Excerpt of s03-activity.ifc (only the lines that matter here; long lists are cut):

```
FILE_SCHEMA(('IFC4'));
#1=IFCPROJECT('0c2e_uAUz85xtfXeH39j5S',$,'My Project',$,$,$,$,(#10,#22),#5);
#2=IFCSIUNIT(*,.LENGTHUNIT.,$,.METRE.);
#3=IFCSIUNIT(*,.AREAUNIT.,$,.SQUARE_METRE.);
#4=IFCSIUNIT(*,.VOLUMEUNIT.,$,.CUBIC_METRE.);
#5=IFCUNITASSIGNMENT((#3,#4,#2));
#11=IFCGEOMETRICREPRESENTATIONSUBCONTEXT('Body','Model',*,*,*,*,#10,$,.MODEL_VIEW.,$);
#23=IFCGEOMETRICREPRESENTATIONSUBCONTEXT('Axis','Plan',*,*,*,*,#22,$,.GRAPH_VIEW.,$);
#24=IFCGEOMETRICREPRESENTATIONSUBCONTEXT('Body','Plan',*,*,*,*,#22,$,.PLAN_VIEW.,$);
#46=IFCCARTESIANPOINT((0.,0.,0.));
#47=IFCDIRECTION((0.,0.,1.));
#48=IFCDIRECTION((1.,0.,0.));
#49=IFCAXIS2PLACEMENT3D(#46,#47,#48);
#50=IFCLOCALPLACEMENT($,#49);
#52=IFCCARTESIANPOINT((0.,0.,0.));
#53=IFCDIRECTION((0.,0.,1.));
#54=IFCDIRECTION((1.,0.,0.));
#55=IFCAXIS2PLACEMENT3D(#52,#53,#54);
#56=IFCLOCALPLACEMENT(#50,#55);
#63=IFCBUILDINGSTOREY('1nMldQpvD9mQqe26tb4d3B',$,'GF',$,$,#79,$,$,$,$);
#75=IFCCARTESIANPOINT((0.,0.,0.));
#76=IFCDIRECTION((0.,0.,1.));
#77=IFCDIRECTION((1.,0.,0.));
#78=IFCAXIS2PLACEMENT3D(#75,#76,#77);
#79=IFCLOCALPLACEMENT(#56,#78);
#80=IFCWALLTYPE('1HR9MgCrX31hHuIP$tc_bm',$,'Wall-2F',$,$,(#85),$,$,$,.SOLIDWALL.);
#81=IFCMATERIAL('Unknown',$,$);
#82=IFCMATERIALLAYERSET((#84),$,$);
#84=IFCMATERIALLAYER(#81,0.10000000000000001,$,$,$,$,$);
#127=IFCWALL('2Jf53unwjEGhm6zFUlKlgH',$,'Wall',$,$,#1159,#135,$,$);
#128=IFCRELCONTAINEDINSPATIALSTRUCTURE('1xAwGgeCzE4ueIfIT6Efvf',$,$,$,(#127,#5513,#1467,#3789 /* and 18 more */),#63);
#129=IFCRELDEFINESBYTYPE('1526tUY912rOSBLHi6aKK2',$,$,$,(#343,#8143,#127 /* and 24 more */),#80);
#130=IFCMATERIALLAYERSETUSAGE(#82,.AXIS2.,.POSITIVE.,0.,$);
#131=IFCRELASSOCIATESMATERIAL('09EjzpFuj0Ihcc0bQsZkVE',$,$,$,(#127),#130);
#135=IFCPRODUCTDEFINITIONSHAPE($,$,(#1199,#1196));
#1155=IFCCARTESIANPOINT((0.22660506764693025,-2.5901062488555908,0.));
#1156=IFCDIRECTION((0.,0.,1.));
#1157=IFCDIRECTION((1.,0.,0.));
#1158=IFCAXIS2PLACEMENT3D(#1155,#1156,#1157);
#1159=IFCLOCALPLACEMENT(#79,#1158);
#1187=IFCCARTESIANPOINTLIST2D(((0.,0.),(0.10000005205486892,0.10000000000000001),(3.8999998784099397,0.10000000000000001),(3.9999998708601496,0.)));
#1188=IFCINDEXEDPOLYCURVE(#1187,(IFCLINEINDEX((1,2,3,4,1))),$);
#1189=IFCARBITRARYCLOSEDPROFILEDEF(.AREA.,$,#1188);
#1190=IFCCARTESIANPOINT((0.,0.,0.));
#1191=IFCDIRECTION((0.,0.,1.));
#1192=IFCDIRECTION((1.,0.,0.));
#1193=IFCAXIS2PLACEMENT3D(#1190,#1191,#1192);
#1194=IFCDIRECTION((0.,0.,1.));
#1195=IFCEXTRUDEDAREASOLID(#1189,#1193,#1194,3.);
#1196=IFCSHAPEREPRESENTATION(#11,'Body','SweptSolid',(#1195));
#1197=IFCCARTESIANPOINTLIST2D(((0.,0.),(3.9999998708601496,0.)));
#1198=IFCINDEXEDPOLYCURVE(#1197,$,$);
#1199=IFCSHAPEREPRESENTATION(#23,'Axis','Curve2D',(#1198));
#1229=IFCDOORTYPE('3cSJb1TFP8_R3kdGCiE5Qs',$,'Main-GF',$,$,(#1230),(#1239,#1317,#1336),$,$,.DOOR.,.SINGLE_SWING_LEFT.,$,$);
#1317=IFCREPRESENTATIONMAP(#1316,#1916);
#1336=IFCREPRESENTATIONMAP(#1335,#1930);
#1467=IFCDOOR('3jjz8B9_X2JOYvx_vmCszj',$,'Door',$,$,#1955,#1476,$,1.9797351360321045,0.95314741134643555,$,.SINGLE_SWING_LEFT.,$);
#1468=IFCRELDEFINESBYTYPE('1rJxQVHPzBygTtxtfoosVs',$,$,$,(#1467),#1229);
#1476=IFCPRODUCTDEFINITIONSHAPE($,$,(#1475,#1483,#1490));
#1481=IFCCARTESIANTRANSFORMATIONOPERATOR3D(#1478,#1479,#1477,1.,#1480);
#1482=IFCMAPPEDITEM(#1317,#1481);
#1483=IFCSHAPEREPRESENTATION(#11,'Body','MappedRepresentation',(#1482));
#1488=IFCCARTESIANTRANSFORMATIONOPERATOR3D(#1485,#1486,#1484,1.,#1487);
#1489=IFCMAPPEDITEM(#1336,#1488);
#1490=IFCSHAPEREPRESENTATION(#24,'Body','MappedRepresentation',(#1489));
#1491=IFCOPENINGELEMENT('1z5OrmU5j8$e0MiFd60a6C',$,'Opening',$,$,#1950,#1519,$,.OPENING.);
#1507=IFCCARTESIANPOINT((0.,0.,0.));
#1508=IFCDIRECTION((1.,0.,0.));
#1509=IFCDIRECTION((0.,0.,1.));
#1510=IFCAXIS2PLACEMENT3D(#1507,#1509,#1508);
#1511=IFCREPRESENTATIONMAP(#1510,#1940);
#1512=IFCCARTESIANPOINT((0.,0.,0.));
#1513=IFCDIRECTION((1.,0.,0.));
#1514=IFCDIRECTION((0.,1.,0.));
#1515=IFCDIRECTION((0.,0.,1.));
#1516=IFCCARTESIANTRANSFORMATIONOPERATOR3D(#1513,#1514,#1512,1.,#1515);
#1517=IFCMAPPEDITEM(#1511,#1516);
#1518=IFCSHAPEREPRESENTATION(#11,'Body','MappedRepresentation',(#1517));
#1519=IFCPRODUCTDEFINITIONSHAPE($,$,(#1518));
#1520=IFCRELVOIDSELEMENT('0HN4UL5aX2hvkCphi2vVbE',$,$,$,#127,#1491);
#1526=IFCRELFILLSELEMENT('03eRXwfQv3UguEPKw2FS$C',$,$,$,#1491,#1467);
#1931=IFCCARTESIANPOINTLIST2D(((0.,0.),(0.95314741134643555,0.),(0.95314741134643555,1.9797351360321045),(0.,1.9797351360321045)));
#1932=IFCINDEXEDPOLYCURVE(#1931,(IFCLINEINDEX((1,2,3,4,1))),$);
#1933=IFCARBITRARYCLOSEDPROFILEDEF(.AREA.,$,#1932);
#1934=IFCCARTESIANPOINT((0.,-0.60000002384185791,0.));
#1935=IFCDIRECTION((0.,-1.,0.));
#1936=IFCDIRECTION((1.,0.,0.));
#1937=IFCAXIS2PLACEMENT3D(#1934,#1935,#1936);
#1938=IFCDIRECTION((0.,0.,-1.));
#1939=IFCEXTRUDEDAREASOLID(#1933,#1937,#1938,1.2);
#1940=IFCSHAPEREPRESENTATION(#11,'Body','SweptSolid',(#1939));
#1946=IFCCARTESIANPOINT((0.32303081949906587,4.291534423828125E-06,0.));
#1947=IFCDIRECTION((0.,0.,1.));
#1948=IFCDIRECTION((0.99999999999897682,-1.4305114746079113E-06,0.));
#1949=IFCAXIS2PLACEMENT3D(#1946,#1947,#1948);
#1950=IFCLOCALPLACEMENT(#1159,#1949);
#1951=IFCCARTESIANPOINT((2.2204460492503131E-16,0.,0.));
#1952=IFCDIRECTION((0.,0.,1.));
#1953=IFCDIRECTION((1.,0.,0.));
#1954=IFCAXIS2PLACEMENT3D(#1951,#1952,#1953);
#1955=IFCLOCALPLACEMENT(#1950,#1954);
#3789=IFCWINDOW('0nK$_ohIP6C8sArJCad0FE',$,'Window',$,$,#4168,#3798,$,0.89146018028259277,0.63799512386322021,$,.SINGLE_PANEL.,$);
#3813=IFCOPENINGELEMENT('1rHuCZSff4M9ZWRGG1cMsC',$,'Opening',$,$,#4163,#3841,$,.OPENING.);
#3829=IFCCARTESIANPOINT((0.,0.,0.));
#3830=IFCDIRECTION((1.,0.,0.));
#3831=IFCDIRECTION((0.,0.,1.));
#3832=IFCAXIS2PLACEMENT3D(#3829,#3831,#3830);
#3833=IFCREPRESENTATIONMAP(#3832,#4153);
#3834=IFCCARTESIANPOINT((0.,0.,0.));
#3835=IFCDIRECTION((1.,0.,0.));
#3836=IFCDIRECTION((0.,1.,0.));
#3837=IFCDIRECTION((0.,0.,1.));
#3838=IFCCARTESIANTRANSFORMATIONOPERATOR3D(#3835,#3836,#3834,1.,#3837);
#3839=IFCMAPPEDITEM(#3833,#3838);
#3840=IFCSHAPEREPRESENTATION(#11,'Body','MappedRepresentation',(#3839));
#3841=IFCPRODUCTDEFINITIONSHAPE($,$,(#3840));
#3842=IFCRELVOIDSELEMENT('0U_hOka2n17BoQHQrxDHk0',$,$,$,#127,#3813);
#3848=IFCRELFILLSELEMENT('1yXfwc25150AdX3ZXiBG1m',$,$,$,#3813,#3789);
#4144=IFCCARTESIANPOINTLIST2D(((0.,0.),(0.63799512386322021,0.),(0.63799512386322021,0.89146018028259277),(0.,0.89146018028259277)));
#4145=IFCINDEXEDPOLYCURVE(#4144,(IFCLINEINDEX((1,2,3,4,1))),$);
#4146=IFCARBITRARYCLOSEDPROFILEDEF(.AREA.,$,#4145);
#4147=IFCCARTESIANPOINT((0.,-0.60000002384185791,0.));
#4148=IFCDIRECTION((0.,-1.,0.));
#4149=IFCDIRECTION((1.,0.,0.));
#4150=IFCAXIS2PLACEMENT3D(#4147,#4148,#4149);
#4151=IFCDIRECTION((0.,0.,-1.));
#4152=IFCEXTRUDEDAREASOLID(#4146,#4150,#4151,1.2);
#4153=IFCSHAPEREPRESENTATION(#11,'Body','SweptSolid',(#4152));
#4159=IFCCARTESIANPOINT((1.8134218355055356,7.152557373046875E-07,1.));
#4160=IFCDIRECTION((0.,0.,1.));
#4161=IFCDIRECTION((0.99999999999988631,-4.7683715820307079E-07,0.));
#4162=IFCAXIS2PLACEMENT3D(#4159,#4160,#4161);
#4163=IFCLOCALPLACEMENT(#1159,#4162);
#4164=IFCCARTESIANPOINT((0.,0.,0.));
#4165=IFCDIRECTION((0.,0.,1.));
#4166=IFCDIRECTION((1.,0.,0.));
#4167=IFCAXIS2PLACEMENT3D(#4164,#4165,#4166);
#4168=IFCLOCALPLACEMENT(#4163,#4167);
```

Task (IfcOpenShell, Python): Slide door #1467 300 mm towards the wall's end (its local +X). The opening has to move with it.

```python
import ifcopenshell
import ifcopenshell.api.geometry
import ifcopenshell.util.placement

model = ifcopenshell.open("s03-activity.ifc")

door = model.by_id(1467)
opening = door.FillsVoids[0].RelatingOpeningElement
wall = opening.VoidsElements[0].RelatingBuildingElement

wall_matrix = ifcopenshell.util.placement.get_local_placement(wall.ObjectPlacement)
shift = wall_matrix[:3, 0] * 0.3
before = ifcopenshell.util.placement.get_local_placement(door.ObjectPlacement)[:3, 3].copy()

# The door is placed relative to its opening, so it follows when the opening moves.
matrix = ifcopenshell.util.placement.get_local_placement(opening.ObjectPlacement)
matrix[:3, 3] += shift
ifcopenshell.api.geometry.edit_object_placement(
    model, product=opening, matrix=matrix, is_si=False, should_transform_children=True
)

after = ifcopenshell.util.placement.get_local_placement(door.ObjectPlacement)[:3, 3]
print("door moved by", (after - before).round(3) + 0.0)

model.write("s03-activity_rev.ifc")
```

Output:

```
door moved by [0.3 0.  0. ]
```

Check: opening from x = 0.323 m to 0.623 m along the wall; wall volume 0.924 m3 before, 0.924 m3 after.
